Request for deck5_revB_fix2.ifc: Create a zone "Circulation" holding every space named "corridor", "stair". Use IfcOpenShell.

First a look at what the model holds.

```python
import ifcopenshell

model = ifcopenshell.open("deck5_revB_fix2.ifc")
print(model.schema)
seen = {}
for space in model.by_type("IfcSpace"):
    seen[space.LongName] = seen.get(space.LongName, 0) + 1
for name, count in sorted(seen.items(), key=str):
    print(count, "x", name)
print("zones:", [z.Name for z in model.by_type("IfcZone")][:20])
```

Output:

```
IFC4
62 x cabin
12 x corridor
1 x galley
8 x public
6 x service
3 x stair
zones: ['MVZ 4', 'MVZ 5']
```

```python
import ifcopenshell
import ifcopenshell.api.group
import ifcopenshell.api.root

model = ifcopenshell.open("deck5_revB_fix2.ifc")

names = {"corridor", "stair"}
spaces = [s for s in model.by_type("IfcSpace") if s.LongName in names]

zone = ifcopenshell.api.root.create_entity(model, ifc_class="IfcZone", name="Circulation")
ifcopenshell.api.group.assign_group(model, products=spaces, group=zone)
print(len(spaces), "spaces in", zone.Name)

model.write("deck5_revB_fix2_updated.ifc")
```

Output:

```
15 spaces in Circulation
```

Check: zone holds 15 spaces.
